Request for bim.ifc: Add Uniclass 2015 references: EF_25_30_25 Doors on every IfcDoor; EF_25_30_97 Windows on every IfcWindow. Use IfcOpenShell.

First a look at what the model holds.

```python
import ifcopenshell

model = ifcopenshell.open("bim.ifc")
print(model.schema)
print("classifications:", [c.Name for c in model.by_type("IfcClassification")])
for ifc_class in ("IfcDoor", "IfcRoof", "IfcStair", "IfcWall", "IfcWindow"):
    print(ifc_class, len(model.by_type(ifc_class)))
```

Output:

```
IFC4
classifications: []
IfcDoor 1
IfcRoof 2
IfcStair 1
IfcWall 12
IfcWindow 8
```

```python
import ifcopenshell
import ifcopenshell.api.classification

model = ifcopenshell.open("bim.ifc")

system = ifcopenshell.api.classification.add_classification(model, classification="Uniclass 2015")

codes = {
    "IfcDoor": ("EF_25_30_25", "Doors"),
    "IfcWindow": ("EF_25_30_97", "Windows"),
}
for ifc_class, (code, name) in codes.items():
    products = model.by_type(ifc_class)
    ifcopenshell.api.classification.add_reference(
        model, products=products, classification=system, identification=code, name=name
    )
    print(code, len(products))

model.write("bim_v2.ifc")
```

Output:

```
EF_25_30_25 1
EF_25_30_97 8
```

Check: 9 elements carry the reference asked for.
